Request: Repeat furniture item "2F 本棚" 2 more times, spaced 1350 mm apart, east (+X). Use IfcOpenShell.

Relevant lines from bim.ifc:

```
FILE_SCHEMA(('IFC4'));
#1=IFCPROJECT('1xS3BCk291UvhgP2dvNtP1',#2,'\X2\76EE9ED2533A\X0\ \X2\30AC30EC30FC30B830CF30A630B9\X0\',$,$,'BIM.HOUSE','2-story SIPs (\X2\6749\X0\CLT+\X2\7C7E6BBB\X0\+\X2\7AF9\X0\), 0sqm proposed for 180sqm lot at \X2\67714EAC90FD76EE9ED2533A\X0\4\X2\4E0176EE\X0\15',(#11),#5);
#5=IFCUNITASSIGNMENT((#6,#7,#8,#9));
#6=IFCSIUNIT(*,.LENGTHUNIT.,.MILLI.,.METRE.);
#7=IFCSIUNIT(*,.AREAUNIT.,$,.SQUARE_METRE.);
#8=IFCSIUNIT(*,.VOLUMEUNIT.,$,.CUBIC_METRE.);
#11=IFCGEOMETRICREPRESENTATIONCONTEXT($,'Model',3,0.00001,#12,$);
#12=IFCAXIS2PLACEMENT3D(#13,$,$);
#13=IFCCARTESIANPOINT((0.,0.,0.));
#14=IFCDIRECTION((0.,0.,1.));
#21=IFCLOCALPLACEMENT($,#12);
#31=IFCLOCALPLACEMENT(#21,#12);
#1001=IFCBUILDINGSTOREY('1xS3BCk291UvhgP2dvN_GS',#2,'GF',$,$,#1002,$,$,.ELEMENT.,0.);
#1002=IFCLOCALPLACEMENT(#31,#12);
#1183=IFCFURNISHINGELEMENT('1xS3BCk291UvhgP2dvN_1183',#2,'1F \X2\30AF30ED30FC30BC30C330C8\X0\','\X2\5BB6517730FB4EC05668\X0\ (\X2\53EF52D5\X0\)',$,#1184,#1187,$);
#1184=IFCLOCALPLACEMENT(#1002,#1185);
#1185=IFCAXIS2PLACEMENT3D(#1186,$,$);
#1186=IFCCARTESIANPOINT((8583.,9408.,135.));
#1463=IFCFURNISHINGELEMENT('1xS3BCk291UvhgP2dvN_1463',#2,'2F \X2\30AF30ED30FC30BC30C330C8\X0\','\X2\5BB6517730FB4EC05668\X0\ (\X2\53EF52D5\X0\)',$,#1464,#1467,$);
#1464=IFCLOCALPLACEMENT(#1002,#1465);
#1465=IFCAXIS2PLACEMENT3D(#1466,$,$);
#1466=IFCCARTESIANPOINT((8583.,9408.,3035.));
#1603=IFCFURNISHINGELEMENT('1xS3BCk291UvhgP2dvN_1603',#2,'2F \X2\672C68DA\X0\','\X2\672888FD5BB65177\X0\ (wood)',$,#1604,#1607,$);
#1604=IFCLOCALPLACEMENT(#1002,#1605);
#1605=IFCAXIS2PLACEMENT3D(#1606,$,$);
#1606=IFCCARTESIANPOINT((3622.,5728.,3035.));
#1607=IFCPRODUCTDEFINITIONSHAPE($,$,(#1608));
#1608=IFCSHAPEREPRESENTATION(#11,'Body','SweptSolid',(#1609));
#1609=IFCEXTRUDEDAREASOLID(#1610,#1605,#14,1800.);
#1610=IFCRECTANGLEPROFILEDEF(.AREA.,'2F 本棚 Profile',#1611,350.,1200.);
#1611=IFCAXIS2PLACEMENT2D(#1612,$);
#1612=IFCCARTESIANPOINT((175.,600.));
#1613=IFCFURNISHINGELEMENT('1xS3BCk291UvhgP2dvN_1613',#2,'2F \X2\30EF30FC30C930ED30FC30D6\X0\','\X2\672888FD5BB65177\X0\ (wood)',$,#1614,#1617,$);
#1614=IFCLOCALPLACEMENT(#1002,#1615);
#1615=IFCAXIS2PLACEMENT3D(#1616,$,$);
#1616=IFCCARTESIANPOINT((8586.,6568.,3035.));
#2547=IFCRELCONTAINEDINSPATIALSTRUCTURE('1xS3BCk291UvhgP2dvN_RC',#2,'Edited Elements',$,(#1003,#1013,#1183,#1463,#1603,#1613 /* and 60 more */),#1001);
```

```python
import numpy as np
import ifcopenshell
import ifcopenshell.api.geometry
import ifcopenshell.api.root
import ifcopenshell.util.element
import ifcopenshell.util.placement
import ifcopenshell.util.unit

model = ifcopenshell.open("bim.ifc")
unit_scale = ifcopenshell.util.unit.calculate_unit_scale(model)


def reuse_history(source, copy):
    """copy_class also copies each property set's owner history, people and application; keep the originals."""
    for rel in copy.IsDefinedBy:
        if rel.is_a("IfcRelDefinesByProperties") and (history := rel.RelatingPropertyDefinition.OwnerHistory):
            rel.RelatingPropertyDefinition.OwnerHistory = source.OwnerHistory
            ifcopenshell.util.element.remove_deep2(model, history)


source = model.by_guid("1xS3BCk291UvhgP2dvN_1603")
base = ifcopenshell.util.placement.get_local_placement(source.ObjectPlacement)
step = np.array([1.0, 0.0, 0.0]) * 1.35 / unit_scale

for i in range(1, 3):
    copy = ifcopenshell.api.root.copy_class(model, product=source)
    copy.Representation = ifcopenshell.util.element.copy_deep(
        model, source.Representation, exclude=["IfcGeometricRepresentationContext", "IfcRepresentationMap"]
    )
    reuse_history(source, copy)
    matrix = base.copy()
    matrix[:3, 3] += i * step
    print("added at", matrix[:3, 3].round(3) + 0.0)
    ifcopenshell.api.geometry.edit_object_placement(model, product=copy, matrix=matrix, is_si=False)

model.write("bim_v2.ifc")
```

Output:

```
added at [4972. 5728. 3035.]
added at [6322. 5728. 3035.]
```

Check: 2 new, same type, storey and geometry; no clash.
